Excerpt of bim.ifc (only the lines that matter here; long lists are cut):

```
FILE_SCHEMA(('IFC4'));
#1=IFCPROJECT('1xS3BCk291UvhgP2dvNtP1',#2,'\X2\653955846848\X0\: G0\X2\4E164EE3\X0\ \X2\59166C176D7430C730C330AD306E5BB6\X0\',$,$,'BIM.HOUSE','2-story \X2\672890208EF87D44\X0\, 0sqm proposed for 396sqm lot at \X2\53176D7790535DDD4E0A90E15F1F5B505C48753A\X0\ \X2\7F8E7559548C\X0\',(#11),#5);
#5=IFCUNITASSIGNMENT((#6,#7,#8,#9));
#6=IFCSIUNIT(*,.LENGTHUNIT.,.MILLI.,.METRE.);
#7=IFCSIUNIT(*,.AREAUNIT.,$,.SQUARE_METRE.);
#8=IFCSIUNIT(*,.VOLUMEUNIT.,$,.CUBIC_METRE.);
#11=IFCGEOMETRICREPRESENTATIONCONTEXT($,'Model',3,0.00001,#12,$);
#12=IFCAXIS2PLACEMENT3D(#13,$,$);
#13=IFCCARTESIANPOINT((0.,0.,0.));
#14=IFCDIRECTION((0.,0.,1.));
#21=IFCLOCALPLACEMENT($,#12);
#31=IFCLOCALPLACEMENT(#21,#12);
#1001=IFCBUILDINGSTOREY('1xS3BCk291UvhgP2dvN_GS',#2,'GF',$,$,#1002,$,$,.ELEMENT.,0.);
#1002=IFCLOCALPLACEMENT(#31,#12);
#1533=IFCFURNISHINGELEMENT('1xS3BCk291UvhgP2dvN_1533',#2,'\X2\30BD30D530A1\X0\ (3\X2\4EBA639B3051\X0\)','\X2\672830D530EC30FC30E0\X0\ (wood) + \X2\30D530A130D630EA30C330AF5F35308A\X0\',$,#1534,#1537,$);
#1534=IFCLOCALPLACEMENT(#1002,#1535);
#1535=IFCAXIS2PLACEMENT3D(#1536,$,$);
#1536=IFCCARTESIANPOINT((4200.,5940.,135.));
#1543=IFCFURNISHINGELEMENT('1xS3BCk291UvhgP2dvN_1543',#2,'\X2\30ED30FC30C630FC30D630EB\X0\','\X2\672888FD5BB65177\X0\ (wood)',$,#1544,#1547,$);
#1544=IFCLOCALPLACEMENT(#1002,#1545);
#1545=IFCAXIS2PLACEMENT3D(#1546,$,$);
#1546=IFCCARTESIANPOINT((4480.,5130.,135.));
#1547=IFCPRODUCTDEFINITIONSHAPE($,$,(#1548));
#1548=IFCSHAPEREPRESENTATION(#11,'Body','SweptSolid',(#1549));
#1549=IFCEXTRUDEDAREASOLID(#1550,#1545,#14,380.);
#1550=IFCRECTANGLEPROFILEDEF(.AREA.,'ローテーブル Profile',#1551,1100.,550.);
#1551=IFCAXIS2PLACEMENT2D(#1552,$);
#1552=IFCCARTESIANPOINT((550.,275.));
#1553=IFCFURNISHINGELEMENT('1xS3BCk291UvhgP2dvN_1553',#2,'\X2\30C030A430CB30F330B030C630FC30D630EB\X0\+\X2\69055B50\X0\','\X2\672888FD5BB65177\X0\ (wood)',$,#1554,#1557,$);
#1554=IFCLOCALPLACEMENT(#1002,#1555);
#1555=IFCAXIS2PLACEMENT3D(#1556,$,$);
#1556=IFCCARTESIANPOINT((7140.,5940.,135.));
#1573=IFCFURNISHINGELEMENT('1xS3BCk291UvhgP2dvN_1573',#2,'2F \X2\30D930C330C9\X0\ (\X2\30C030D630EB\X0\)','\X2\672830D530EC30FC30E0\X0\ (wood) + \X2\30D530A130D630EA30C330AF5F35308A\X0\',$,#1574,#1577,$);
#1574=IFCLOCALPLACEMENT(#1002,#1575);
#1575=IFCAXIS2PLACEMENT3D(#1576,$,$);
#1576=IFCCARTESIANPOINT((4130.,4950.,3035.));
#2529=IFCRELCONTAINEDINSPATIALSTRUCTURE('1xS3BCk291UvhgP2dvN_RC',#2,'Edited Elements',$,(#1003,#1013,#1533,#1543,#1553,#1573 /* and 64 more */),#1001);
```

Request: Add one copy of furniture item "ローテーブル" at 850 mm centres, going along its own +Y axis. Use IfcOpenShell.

```python
import ifcopenshell
import ifcopenshell.api.geometry
import ifcopenshell.api.root
import ifcopenshell.util.element
import ifcopenshell.util.placement
import ifcopenshell.util.unit

model = ifcopenshell.open("bim.ifc")
unit_scale = ifcopenshell.util.unit.calculate_unit_scale(model)


def reuse_history(source, copy):
    """copy_class also copies each property set's owner history, people and application; keep the originals."""
    for rel in copy.IsDefinedBy:
        if rel.is_a("IfcRelDefinesByProperties") and (history := rel.RelatingPropertyDefinition.OwnerHistory):
            rel.RelatingPropertyDefinition.OwnerHistory = source.OwnerHistory
            ifcopenshell.util.element.remove_deep2(model, history)


source = model.by_id(1543)
base = ifcopenshell.util.placement.get_local_placement(source.ObjectPlacement)
step = base[:3, 1] * 0.85 / unit_scale

for i in range(1, 2):
    copy = ifcopenshell.api.root.copy_class(model, product=source)
    copy.Representation = ifcopenshell.util.element.copy_deep(
        model, source.Representation, exclude=["IfcGeometricRepresentationContext", "IfcRepresentationMap"]
    )
    reuse_history(source, copy)
    matrix = base.copy()
    matrix[:3, 3] += i * step
    print("added at", matrix[:3, 3].round(3) + 0.0)
    ifcopenshell.api.geometry.edit_object_placement(model, product=copy, matrix=matrix, is_si=False)

model.write("bim-out.ifc")
```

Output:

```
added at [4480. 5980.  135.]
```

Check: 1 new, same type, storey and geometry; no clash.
